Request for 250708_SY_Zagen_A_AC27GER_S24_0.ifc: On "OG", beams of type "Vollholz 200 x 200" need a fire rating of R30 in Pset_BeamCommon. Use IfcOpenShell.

First a look at what the model holds.

```python
import ifcopenshell
import ifcopenshell.util.element

model = ifcopenshell.open("250708_SY_Zagen_A_AC27GER_S24_0.ifc")
print(model.schema)
storey = next(s for s in model.by_type("IfcBuildingStorey") if s.Name == "OG")
beams = [e for e in ifcopenshell.util.element.get_decomposition(storey) if e.is_a("IfcBeam")]
seen = {}
for e in beams:
    element_type = ifcopenshell.util.element.get_type(e)
    key = (element_type.Name if element_type != e and element_type else None, ifcopenshell.util.element.get_pset(e, "Pset_BeamCommon", "FireRating"))
    seen[key] = seen.get(key, 0) + 1
for (name, value), count in sorted(seen.items(), key=str):
    print(count, "x", name, "|", value)
```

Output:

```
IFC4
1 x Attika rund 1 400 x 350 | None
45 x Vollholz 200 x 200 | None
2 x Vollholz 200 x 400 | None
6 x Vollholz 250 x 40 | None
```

```python
import ifcopenshell
import ifcopenshell.api.pset
import ifcopenshell.util.element

model = ifcopenshell.open("250708_SY_Zagen_A_AC27GER_S24_0.ifc")

storey = next(s for s in model.by_type("IfcBuildingStorey") if s.Name == "OG")
beams = [e for e in ifcopenshell.util.element.get_decomposition(storey) if e.is_a("IfcBeam")]

count = 0
for e in beams:
    element_type = ifcopenshell.util.element.get_type(e)
    if element_type in (None, e) or element_type.Name != "Vollholz 200 x 200":
        continue
    # add_pset returns the element's existing set when there is one.
    pset = ifcopenshell.api.pset.add_pset(model, product=e, name="Pset_BeamCommon")
    ifcopenshell.api.pset.edit_pset(model, pset=pset, properties={"FireRating": "R30"})
    count += 1

print(count, "beams updated")

model.write("250708_SY_Zagen_A_AC27GER_S24_0_v2.ifc")
```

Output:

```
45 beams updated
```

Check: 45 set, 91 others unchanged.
